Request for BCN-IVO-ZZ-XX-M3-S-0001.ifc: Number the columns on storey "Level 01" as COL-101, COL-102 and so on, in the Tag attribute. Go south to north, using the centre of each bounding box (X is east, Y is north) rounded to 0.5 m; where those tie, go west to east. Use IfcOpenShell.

First a look at what the model holds.

```python
import ifcopenshell
import ifcopenshell.util.element
import ifcopenshell.util.placement

model = ifcopenshell.open("BCN-IVO-ZZ-XX-M3-S-0001.ifc")
print(model.schema)
storey = next(s for s in model.by_type("IfcBuildingStorey") if s.Name == "Level 01")
columns = [e for e in ifcopenshell.util.element.get_decomposition(storey) if e.is_a("IfcColumn")]
for e in sorted(columns, key=lambda e: e.id()):
    origin = ifcopenshell.util.placement.get_local_placement(e.ObjectPlacement)[:3, 3]
    print(e.id(), e.Tag, e.Name, origin.round(2) + 0.0, sep=" | ")
```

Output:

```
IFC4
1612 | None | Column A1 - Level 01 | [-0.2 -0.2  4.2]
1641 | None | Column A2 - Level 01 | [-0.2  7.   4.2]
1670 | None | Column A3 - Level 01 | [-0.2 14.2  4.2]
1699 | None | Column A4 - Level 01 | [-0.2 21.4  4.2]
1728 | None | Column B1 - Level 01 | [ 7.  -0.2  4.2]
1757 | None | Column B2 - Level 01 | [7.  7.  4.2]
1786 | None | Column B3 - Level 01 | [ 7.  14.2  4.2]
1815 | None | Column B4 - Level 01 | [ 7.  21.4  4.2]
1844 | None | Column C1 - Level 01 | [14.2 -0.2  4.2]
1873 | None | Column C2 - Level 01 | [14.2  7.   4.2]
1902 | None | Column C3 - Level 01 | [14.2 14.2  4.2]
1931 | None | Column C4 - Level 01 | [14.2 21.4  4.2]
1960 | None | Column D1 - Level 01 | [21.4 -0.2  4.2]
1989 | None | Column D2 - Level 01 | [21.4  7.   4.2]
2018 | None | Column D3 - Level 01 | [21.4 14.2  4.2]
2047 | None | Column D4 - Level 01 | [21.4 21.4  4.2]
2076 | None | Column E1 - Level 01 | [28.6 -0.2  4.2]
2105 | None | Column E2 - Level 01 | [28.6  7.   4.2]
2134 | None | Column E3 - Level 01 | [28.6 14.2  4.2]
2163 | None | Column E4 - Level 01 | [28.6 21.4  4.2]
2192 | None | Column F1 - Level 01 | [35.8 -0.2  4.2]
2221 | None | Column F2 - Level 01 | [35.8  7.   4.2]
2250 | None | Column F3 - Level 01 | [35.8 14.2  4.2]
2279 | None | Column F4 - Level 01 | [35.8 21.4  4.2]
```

```python
import ifcopenshell
import ifcopenshell.geom
import ifcopenshell.util.element
import ifcopenshell.util.shape

model = ifcopenshell.open("BCN-IVO-ZZ-XX-M3-S-0001.ifc")
settings = ifcopenshell.geom.settings()
settings.set("use-world-coords", True)


def centre(element):
    shape = ifcopenshell.geom.create_shape(settings, element)
    return ifcopenshell.util.shape.get_bbox_centroid(shape.geometry)


storey = next(s for s in model.by_type("IfcBuildingStorey") if s.Name == "Level 01")
columns = [e for e in ifcopenshell.util.element.get_decomposition(storey) if e.is_a("IfcColumn")]

# Insertion points can sit at a corner or the storey origin, so sort by the geometry (in metres).
centres = {e: centre(e) for e in columns}
columns.sort(key=lambda e: (round(centres[e][1] / 0.5), centres[e][0]))

for i, e in enumerate(columns, start=1):
    number = f"COL-1{i:02d}"
    e.Tag = number
    print(e.id(), number)

model.write("BCN-IVO-ZZ-XX-M3-S-0001_v2.ifc")
```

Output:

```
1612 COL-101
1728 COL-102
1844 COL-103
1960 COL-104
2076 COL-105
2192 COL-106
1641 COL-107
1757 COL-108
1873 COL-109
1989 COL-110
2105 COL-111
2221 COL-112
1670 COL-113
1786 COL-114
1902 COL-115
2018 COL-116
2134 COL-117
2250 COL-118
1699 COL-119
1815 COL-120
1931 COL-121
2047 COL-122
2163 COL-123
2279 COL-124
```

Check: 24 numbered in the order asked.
